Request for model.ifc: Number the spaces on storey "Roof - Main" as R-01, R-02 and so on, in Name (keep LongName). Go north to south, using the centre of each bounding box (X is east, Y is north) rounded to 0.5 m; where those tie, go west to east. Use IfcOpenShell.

First a look at what the model holds.

```python
import ifcopenshell
import ifcopenshell.util.element
import ifcopenshell.util.placement

model = ifcopenshell.open("model.ifc")
print(model.schema)
storey = next(s for s in model.by_type("IfcBuildingStorey") if s.Name == "Roof - Main")
spaces = [e for e in ifcopenshell.util.element.get_decomposition(storey) if e.is_a("IfcSpace")]
for e in sorted(spaces, key=lambda e: e.id()):
    origin = ifcopenshell.util.placement.get_local_placement(e.ObjectPlacement)[:3, 3]
    print(e.id(), e.Name, e.LongName, origin.round(2) + 0.0, sep=" | ")
```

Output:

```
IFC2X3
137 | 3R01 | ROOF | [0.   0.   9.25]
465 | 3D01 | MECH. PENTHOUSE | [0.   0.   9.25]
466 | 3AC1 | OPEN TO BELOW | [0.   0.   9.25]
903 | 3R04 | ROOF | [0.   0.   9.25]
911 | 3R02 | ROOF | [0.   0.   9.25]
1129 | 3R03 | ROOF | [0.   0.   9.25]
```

```python
import ifcopenshell
import ifcopenshell.geom
import ifcopenshell.util.element
import ifcopenshell.util.shape

model = ifcopenshell.open("model.ifc")
settings = ifcopenshell.geom.settings()
settings.set("use-world-coords", True)


def centre(element):
    shape = ifcopenshell.geom.create_shape(settings, element)
    return ifcopenshell.util.shape.get_bbox_centroid(shape.geometry)


storey = next(s for s in model.by_type("IfcBuildingStorey") if s.Name == "Roof - Main")
spaces = [e for e in ifcopenshell.util.element.get_decomposition(storey) if e.is_a("IfcSpace")]

# Insertion points can sit at a corner or the storey origin, so sort by the geometry (in metres).
centres = {e: centre(e) for e in spaces}
spaces.sort(key=lambda e: (-round(centres[e][1] / 0.5), centres[e][0]))

for i, e in enumerate(spaces, start=1):
    number = f"R-{i:02d}"
    e.Name = number
    print(e.id(), number)

model.write("model_edited.ifc")
```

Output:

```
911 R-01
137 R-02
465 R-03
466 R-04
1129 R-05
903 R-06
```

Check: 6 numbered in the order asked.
